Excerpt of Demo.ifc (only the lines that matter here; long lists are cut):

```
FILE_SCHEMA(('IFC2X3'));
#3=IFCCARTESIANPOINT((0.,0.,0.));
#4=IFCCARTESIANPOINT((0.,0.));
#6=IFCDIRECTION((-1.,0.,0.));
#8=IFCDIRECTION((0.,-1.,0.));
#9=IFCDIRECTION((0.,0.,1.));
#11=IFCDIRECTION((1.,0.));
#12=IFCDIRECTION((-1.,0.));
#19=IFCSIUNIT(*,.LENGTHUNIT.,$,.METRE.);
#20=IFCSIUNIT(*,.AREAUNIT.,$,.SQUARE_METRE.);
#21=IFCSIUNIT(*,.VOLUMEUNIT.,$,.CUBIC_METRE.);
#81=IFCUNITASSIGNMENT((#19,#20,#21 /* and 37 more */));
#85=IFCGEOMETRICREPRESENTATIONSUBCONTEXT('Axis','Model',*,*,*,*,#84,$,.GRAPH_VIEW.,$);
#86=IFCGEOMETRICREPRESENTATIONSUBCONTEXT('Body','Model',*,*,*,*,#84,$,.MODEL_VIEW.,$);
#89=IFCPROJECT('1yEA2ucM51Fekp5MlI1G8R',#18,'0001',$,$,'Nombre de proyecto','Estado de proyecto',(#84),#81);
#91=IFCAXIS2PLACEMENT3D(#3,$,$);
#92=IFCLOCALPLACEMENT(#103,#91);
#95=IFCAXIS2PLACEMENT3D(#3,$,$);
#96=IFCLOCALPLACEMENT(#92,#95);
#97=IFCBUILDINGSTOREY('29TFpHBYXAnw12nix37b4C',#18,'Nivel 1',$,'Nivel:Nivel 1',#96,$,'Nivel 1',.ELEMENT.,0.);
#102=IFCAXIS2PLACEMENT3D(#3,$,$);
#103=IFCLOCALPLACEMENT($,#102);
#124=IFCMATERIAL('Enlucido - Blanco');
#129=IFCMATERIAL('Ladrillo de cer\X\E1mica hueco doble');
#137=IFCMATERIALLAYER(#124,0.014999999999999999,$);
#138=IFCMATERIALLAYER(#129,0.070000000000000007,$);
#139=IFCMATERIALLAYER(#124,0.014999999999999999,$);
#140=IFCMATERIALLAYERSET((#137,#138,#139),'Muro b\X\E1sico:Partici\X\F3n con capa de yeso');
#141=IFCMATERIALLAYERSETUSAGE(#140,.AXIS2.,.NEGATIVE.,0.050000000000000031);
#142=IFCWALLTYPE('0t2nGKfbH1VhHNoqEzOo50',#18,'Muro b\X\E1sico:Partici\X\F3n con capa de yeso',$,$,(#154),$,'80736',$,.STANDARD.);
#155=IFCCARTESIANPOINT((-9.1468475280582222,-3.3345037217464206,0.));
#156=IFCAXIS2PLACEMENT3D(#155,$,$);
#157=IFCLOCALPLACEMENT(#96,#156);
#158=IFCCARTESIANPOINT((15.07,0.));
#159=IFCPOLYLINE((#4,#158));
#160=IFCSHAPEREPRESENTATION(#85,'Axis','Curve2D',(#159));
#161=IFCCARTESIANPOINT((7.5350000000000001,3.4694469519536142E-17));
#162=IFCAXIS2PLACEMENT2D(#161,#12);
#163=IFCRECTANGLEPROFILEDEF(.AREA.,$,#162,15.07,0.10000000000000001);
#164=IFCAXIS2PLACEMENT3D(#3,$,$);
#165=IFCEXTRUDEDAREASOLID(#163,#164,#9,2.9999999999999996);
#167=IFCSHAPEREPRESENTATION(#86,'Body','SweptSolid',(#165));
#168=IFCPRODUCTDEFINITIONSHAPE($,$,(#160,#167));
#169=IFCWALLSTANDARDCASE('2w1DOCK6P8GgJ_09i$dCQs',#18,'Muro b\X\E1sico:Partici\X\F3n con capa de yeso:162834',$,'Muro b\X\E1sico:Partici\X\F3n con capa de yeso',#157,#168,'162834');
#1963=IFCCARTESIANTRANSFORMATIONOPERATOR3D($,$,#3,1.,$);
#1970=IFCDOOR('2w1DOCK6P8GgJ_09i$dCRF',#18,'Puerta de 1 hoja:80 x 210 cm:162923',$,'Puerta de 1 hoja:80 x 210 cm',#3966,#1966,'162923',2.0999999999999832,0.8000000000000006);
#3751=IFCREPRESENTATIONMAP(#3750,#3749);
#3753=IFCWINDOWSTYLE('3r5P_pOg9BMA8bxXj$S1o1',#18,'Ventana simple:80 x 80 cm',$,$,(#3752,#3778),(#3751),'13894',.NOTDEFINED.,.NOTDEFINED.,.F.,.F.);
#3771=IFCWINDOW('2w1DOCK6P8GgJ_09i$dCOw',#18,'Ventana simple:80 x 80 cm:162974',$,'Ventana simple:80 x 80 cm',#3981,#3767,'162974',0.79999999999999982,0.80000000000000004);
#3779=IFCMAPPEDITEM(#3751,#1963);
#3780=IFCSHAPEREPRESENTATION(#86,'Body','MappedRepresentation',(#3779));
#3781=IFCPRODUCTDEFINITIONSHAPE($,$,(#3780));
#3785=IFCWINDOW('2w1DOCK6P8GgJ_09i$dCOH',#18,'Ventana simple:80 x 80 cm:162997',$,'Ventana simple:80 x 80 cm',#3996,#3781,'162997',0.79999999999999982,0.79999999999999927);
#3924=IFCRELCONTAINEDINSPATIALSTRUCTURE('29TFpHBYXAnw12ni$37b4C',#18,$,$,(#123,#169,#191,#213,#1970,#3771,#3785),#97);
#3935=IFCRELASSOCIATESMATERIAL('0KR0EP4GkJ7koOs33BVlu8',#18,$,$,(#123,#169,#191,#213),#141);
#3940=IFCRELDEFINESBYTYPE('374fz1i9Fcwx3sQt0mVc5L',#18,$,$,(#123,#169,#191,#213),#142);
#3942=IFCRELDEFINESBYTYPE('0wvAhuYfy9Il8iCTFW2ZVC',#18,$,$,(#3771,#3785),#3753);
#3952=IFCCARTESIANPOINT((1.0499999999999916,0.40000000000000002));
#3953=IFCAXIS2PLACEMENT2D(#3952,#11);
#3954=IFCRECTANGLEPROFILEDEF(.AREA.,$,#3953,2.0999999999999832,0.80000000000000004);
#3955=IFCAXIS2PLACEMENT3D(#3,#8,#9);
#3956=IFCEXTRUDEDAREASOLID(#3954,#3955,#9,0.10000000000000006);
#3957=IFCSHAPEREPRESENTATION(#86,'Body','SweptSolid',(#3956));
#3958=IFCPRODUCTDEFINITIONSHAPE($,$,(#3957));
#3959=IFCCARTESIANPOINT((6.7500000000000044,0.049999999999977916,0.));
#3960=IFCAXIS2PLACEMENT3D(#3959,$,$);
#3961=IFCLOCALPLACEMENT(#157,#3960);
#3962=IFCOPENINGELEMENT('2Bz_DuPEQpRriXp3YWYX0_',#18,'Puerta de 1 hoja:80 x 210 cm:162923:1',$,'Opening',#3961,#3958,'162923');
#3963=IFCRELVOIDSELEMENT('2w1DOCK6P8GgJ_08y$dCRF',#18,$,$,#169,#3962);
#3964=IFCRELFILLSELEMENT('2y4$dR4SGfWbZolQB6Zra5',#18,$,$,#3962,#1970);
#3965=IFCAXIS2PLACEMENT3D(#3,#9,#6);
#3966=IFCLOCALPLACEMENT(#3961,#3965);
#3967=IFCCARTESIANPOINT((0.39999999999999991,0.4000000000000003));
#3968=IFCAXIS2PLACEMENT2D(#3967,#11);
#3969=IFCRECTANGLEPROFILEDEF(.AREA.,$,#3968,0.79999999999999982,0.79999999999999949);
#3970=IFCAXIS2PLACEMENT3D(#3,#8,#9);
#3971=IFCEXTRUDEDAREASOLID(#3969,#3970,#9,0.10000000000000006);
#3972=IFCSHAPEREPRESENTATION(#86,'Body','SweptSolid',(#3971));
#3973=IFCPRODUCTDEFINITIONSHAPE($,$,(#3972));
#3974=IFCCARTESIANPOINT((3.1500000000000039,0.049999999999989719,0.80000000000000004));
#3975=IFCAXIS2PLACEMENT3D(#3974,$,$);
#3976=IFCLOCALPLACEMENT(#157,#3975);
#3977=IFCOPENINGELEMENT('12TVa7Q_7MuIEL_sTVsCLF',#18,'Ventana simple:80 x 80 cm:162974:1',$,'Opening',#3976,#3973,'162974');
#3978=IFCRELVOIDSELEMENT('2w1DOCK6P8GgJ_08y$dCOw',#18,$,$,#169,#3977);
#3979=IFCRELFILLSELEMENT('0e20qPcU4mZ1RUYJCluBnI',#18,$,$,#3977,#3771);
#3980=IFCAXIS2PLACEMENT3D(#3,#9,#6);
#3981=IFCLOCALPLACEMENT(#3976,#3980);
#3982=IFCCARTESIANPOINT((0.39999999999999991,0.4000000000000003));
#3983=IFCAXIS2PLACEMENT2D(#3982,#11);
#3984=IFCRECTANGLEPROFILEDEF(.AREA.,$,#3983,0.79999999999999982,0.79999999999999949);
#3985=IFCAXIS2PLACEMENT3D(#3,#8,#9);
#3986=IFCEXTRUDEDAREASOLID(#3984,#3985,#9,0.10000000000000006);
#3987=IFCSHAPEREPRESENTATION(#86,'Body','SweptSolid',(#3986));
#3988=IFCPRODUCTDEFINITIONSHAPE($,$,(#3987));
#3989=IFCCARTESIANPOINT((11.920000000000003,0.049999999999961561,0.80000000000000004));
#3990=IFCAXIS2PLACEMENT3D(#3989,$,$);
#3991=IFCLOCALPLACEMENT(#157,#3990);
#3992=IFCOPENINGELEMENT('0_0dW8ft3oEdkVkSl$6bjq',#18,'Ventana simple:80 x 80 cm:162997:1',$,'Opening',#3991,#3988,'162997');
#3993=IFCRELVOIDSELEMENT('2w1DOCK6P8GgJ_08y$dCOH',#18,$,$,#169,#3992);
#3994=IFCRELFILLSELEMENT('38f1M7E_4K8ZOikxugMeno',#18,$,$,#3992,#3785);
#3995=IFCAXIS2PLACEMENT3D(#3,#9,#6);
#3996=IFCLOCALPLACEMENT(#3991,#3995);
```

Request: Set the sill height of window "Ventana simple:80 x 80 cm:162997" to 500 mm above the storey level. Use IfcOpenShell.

```python
import numpy as np
import ifcopenshell
import ifcopenshell.api.geometry
import ifcopenshell.geom
import ifcopenshell.util.element
import ifcopenshell.util.placement
import ifcopenshell.util.shape
import ifcopenshell.util.unit

model = ifcopenshell.open("Demo.ifc")
unit_scale = ifcopenshell.util.unit.calculate_unit_scale(model)

window = model.by_guid("2w1DOCK6P8GgJ_09i$dCOH")
opening = window.FillsVoids[0].RelatingOpeningElement
storey = ifcopenshell.util.element.get_container(window, ifc_class="IfcBuildingStorey")
level = ifcopenshell.util.placement.get_local_placement(storey.ObjectPlacement)[2, 3]

# The opening's origin need not be at the sill, so measure its lowest point.
shape = ifcopenshell.geom.create_shape(ifcopenshell.geom.settings(), opening)
bottom = ifcopenshell.util.shape.get_shape_bottom_elevation(shape, shape.geometry) / unit_scale
dz = level + 0.5 / unit_scale - bottom

shift = np.array([0.0, 0.0, dz])
# The window is placed relative to its opening, so it follows when the opening moves.
matrix = ifcopenshell.util.placement.get_local_placement(opening.ObjectPlacement)
matrix[:3, 3] += shift
ifcopenshell.api.geometry.edit_object_placement(
    model, product=opening, matrix=matrix, is_si=False, should_transform_children=True
)

print(f"moved by {dz * unit_scale:+.3f} m")

model.write("Demo_rev.ifc")
```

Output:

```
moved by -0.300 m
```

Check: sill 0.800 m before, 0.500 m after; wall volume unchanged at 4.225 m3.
